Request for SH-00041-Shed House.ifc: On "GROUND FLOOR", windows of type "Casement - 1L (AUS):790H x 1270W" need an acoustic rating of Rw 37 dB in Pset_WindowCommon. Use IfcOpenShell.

First a look at what the model holds.

```python
import ifcopenshell
import ifcopenshell.util.element

model = ifcopenshell.open("SH-00041-Shed House.ifc")
print(model.schema)
storey = next(s for s in model.by_type("IfcBuildingStorey") if s.Name == "GROUND FLOOR")
windows = [e for e in ifcopenshell.util.element.get_decomposition(storey) if e.is_a("IfcWindow")]
seen = {}
for e in windows:
    element_type = ifcopenshell.util.element.get_type(e)
    key = (element_type.Name if element_type != e and element_type else None, ifcopenshell.util.element.get_pset(e, "Pset_WindowCommon", "AcousticRating"))
    seen[key] = seen.get(key, 0) + 1
for (name, value), count in sorted(seen.items(), key=str):
    print(count, "x", name, "|", value)
```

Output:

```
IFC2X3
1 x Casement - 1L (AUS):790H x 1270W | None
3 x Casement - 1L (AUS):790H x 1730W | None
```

```python
import ifcopenshell
import ifcopenshell.api.pset
import ifcopenshell.util.element

model = ifcopenshell.open("SH-00041-Shed House.ifc")

storey = next(s for s in model.by_type("IfcBuildingStorey") if s.Name == "GROUND FLOOR")
windows = [e for e in ifcopenshell.util.element.get_decomposition(storey) if e.is_a("IfcWindow")]

count = 0
for e in windows:
    element_type = ifcopenshell.util.element.get_type(e)
    if element_type in (None, e) or element_type.Name != "Casement - 1L (AUS):790H x 1270W":
        continue
    # add_pset returns the element's existing set when there is one.
    pset = ifcopenshell.api.pset.add_pset(model, product=e, name="Pset_WindowCommon")
    ifcopenshell.api.pset.edit_pset(model, pset=pset, properties={"AcousticRating": "Rw 37 dB"})
    count += 1

print(count, "windows updated")

model.write("SH-00041-Shed House_updated.ifc")
```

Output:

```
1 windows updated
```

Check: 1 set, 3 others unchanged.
